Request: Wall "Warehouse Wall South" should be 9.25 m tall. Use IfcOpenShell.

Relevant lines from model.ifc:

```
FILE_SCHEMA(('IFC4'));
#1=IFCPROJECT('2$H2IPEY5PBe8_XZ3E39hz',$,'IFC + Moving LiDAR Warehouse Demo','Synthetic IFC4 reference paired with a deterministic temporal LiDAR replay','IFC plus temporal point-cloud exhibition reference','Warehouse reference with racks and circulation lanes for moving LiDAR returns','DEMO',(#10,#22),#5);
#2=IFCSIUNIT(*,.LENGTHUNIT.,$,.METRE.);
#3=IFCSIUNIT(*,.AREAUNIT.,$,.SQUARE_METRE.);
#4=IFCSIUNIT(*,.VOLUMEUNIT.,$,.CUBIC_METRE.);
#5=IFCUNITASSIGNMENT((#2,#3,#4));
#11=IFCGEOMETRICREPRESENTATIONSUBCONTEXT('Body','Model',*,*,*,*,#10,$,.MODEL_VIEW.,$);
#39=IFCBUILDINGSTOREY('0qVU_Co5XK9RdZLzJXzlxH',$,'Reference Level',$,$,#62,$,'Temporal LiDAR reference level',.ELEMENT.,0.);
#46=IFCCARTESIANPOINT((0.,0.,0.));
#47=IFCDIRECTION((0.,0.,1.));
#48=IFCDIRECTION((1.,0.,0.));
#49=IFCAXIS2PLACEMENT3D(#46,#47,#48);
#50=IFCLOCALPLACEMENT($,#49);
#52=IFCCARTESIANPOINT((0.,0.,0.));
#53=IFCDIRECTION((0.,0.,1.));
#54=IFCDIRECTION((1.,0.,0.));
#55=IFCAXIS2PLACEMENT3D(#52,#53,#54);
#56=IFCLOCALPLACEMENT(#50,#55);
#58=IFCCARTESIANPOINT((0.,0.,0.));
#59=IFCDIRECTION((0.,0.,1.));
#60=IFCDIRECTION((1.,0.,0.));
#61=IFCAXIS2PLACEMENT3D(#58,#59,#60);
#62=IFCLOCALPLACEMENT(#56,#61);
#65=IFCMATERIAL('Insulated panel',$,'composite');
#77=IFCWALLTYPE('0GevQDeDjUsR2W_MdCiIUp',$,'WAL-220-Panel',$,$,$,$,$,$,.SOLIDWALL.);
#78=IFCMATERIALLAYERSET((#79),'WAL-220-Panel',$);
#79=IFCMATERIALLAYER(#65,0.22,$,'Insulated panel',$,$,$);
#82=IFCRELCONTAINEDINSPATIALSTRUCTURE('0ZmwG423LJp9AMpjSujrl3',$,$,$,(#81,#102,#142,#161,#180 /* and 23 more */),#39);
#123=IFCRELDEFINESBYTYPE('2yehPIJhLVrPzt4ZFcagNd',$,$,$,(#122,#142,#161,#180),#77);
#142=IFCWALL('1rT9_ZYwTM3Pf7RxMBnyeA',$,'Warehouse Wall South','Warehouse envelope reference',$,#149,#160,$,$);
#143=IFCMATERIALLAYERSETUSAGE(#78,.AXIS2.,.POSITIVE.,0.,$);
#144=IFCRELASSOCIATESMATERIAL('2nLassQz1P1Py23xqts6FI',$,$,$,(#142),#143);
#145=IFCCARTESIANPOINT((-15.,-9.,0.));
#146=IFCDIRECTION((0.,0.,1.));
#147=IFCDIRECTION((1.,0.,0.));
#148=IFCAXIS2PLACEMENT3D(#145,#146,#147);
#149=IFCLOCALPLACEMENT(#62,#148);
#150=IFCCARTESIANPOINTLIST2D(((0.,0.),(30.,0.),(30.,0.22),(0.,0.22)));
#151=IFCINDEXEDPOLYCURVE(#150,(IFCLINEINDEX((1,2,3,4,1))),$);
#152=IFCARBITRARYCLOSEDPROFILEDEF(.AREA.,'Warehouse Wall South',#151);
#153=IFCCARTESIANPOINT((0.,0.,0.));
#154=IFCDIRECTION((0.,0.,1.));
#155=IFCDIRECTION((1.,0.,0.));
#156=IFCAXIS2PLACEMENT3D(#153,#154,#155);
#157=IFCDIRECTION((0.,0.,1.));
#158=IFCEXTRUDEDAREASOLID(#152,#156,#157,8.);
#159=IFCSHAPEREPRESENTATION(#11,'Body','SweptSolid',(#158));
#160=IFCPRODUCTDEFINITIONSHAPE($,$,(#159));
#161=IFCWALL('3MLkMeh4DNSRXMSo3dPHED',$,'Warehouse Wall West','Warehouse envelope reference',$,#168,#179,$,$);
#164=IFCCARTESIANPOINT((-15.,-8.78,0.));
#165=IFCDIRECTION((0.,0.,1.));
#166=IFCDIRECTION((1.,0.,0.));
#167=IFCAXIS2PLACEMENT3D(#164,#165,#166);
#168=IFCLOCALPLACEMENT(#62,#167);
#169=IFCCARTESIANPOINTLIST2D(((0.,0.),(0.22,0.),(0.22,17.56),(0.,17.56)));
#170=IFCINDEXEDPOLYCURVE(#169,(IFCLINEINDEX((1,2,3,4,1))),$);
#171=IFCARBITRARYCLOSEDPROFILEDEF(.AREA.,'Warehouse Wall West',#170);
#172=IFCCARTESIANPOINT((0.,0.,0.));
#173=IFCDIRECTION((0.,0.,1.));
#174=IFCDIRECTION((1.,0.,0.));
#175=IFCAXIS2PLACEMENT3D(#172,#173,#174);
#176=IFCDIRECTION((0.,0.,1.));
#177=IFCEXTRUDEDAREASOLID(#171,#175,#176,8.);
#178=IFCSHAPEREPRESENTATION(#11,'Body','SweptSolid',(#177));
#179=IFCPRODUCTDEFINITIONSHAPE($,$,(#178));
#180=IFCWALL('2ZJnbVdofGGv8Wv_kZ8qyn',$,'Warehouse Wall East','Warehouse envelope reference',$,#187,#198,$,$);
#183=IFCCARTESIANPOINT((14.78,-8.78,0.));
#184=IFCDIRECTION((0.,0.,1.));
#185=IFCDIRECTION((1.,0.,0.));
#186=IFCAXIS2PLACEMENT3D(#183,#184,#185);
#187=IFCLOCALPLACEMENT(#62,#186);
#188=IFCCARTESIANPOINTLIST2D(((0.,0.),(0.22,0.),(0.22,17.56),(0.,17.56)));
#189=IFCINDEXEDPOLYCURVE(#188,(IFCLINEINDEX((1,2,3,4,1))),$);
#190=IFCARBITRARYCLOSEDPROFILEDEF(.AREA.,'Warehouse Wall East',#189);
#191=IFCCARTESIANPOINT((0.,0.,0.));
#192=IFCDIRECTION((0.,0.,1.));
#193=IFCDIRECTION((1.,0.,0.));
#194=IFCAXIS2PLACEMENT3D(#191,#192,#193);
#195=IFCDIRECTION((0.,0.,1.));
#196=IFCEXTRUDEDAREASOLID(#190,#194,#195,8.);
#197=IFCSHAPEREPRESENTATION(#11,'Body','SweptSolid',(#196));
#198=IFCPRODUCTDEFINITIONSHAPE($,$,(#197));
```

```python
import ifcopenshell
import ifcopenshell.geom
import ifcopenshell.util.representation
import ifcopenshell.util.shape
import ifcopenshell.util.unit

model = ifcopenshell.open("model.ifc")
unit_scale = ifcopenshell.util.unit.calculate_unit_scale(model)
settings = ifcopenshell.geom.settings()


def volume(element):
    """Net volume in cubic metres, openings subtracted."""
    shape = ifcopenshell.geom.create_shape(settings, element)
    return ifcopenshell.util.shape.get_volume(shape.geometry)


wall = model.by_id(142)
before = volume(wall)

body = ifcopenshell.util.representation.get_representation(wall, "Model", "Body")
solid = body.Items[0]
old_height = solid.Depth
solid.Depth = 9.25 / unit_scale
after = volume(wall)

print(f"height {old_height:g} -> {solid.Depth:g}, volume {before:.3f} -> {after:.3f} m3")

model.write("model_edited.ifc")
```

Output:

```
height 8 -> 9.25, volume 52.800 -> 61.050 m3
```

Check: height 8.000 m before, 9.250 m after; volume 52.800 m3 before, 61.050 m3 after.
